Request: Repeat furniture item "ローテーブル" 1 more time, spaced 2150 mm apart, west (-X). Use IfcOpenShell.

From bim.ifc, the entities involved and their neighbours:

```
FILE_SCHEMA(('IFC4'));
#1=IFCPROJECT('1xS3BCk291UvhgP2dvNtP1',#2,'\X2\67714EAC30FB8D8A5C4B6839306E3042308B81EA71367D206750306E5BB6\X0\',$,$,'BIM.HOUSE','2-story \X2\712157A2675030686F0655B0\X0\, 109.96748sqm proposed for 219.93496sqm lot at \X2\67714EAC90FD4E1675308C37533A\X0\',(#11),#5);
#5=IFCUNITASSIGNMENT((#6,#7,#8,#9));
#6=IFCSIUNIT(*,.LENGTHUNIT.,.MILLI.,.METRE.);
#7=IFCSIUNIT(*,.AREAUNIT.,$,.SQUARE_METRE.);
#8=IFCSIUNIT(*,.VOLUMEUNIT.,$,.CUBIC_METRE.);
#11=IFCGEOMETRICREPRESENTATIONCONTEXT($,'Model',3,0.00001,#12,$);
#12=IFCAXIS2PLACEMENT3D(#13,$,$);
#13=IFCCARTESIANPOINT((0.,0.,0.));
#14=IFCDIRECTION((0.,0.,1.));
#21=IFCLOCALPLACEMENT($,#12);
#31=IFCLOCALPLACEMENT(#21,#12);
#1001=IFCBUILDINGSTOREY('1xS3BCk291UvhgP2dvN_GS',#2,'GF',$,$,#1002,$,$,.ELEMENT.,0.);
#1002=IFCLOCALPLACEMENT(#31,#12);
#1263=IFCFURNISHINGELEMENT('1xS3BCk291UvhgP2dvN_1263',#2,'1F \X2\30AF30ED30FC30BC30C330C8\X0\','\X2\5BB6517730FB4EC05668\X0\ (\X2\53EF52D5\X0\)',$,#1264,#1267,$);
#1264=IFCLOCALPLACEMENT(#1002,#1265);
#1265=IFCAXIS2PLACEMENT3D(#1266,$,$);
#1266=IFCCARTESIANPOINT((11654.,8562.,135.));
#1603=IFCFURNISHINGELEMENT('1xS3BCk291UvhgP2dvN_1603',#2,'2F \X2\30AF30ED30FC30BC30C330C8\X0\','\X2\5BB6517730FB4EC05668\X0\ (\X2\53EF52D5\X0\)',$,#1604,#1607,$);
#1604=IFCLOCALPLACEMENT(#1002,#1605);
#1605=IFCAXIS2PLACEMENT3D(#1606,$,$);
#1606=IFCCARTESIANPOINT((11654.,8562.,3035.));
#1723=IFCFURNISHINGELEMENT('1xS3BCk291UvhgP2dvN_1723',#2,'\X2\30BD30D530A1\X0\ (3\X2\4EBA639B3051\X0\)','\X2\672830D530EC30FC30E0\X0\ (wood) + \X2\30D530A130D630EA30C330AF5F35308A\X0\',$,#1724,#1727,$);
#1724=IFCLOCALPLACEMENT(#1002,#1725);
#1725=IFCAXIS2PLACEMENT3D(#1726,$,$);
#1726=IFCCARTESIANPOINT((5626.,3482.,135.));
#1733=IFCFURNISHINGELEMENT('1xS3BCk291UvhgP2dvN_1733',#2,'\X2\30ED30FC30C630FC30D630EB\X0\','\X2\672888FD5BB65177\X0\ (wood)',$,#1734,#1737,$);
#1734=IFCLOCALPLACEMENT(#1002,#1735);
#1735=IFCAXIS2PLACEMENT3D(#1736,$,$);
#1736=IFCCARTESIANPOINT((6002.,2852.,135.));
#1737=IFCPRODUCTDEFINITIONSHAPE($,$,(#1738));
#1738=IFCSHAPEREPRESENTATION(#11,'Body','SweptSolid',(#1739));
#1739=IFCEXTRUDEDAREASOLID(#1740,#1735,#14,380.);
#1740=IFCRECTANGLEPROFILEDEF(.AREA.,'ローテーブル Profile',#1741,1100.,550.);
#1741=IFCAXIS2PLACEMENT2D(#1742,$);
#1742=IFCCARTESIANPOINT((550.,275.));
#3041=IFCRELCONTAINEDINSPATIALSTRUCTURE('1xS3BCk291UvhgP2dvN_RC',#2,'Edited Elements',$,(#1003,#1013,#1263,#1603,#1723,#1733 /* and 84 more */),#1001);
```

```python
import numpy as np
import ifcopenshell
import ifcopenshell.api.geometry
import ifcopenshell.api.root
import ifcopenshell.util.element
import ifcopenshell.util.placement

model = ifcopenshell.open("bim.ifc")


def reuse_history(source, copy):
    """copy_class also copies each property set's owner history, people and application; keep the originals."""
    for rel in copy.IsDefinedBy:
        if rel.is_a("IfcRelDefinesByProperties") and (history := rel.RelatingPropertyDefinition.OwnerHistory):
            rel.RelatingPropertyDefinition.OwnerHistory = source.OwnerHistory
            ifcopenshell.util.element.remove_deep2(model, history)


source = model.by_guid("1xS3BCk291UvhgP2dvN_1733")
base = ifcopenshell.util.placement.get_local_placement(source.ObjectPlacement)
step = np.array([-1.0, 0.0, 0.0]) * 2150.0

for i in range(1, 2):
    copy = ifcopenshell.api.root.copy_class(model, product=source)
    copy.Representation = ifcopenshell.util.element.copy_deep(
        model, source.Representation, exclude=["IfcGeometricRepresentationContext", "IfcRepresentationMap"]
    )
    reuse_history(source, copy)
    matrix = base.copy()
    matrix[:3, 3] += i * step
    print("added at", matrix[:3, 3].round(3) + 0.0)
    ifcopenshell.api.geometry.edit_object_placement(model, product=copy, matrix=matrix, is_si=False)

model.write("bim_edited.ifc")
```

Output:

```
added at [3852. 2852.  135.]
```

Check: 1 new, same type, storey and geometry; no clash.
